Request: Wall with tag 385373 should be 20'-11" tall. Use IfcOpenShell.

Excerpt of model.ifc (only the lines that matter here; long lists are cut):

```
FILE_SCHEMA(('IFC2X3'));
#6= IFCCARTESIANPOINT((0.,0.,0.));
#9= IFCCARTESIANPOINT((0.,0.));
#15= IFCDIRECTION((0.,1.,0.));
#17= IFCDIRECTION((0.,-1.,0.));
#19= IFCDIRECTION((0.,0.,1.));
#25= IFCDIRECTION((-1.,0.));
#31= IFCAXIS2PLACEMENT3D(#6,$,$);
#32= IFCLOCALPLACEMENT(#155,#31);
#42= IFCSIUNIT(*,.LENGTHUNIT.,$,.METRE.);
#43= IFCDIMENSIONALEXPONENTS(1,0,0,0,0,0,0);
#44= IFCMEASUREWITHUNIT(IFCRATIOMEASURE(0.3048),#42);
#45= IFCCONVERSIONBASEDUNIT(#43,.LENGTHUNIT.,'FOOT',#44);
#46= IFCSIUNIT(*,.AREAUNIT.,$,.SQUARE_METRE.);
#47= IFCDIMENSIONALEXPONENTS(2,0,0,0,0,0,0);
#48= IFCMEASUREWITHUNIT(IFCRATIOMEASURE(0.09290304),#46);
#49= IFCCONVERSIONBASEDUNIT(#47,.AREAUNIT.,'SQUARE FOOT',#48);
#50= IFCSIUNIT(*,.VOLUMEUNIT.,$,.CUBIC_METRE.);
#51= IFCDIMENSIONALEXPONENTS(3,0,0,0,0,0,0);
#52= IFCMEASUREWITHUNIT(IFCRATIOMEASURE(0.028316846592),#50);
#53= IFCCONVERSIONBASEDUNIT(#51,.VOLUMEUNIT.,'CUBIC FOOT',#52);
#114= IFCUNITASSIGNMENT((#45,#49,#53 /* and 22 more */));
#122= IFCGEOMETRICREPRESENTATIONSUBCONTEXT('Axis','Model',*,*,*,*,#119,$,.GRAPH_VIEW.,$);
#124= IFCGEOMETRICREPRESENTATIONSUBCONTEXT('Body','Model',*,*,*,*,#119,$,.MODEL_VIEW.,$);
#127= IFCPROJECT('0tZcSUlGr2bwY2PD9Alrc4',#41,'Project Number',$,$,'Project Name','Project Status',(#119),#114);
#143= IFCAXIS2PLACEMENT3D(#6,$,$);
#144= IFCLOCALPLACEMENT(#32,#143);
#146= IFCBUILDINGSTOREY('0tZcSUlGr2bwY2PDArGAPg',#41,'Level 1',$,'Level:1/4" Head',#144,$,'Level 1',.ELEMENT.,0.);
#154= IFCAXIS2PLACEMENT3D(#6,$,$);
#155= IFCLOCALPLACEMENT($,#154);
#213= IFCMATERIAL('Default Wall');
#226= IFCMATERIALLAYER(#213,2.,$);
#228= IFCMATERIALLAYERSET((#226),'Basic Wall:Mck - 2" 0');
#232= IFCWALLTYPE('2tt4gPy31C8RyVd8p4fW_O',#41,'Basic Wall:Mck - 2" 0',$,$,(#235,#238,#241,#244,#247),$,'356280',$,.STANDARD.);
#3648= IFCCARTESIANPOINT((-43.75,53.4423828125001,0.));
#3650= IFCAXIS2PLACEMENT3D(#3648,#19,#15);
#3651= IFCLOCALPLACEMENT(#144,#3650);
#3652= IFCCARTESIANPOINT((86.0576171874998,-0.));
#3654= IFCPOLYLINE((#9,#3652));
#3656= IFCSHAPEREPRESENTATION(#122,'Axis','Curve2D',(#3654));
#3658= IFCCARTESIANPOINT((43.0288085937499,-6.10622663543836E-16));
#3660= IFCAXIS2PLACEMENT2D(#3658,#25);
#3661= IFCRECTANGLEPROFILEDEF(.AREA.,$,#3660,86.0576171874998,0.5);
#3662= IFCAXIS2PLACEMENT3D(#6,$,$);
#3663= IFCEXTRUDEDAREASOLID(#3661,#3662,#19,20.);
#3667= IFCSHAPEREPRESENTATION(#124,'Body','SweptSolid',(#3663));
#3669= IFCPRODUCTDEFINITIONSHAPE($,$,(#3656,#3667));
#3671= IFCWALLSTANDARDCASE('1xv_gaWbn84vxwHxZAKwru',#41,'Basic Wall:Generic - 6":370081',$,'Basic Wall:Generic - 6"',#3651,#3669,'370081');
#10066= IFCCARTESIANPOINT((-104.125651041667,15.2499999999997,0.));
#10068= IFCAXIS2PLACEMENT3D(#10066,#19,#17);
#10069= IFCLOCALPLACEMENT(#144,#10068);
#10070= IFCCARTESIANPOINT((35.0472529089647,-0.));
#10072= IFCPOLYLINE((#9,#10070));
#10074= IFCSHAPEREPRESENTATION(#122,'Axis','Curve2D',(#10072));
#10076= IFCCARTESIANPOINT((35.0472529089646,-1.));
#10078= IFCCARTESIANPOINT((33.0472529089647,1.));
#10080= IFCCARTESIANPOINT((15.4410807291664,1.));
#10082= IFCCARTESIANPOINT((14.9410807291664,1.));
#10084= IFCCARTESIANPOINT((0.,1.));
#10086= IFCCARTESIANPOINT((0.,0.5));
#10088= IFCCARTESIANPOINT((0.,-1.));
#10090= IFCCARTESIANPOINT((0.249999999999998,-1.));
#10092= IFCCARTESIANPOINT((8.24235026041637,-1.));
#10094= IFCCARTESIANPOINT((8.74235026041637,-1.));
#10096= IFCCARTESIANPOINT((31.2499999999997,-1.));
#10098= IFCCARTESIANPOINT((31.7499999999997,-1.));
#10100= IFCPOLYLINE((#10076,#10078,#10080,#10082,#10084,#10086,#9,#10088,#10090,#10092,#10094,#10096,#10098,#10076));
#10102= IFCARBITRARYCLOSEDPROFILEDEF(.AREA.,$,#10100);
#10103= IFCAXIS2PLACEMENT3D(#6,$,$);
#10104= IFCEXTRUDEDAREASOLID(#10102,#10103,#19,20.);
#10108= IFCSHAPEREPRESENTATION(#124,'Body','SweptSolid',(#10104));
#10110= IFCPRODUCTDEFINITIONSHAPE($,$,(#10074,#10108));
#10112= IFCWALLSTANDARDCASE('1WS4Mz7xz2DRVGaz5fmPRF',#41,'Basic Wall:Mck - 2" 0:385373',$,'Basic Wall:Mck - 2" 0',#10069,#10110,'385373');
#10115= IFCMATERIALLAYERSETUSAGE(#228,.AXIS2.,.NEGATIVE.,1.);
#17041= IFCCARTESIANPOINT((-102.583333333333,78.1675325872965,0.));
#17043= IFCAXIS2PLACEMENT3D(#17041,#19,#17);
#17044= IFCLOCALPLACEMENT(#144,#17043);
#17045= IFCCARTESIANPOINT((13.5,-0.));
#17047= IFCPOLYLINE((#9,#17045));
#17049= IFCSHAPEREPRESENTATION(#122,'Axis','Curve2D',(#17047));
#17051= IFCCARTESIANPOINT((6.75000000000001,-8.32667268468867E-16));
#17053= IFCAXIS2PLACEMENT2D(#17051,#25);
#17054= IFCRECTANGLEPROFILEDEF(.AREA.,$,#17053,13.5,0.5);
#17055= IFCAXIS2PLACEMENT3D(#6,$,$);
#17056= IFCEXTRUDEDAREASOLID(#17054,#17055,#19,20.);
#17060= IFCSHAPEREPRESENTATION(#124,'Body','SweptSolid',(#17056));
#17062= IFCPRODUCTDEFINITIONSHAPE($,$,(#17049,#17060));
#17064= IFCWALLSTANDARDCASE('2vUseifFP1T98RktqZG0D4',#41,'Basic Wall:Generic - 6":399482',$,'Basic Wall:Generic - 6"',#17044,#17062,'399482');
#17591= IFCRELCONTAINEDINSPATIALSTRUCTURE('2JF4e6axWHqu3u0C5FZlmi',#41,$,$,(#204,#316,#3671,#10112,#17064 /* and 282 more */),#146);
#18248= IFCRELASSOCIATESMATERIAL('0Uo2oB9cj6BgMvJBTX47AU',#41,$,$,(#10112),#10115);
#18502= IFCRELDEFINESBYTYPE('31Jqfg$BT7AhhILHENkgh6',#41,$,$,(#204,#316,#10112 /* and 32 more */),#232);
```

```python
import ifcopenshell
import ifcopenshell.geom
import ifcopenshell.util.representation
import ifcopenshell.util.shape
import ifcopenshell.util.unit

model = ifcopenshell.open("model.ifc")
unit_scale = ifcopenshell.util.unit.calculate_unit_scale(model)
settings = ifcopenshell.geom.settings()


def volume(element):
    """Net volume in cubic metres, openings subtracted."""
    shape = ifcopenshell.geom.create_shape(settings, element)
    return ifcopenshell.util.shape.get_volume(shape.geometry)


wall = model.by_guid("1WS4Mz7xz2DRVGaz5fmPRF")
before = volume(wall)

body = ifcopenshell.util.representation.get_representation(wall, "Model", "Body")
solid = body.Items[0]
old_height = solid.Depth
solid.Depth = 251 * 0.0254 / unit_scale
after = volume(wall)

print(f"height {old_height:g} -> {solid.Depth:g}, volume {before:.3f} -> {after:.3f} m3")

model.write("model_v2.ifc")
```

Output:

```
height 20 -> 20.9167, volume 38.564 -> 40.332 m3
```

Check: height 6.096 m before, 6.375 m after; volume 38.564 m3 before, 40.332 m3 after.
